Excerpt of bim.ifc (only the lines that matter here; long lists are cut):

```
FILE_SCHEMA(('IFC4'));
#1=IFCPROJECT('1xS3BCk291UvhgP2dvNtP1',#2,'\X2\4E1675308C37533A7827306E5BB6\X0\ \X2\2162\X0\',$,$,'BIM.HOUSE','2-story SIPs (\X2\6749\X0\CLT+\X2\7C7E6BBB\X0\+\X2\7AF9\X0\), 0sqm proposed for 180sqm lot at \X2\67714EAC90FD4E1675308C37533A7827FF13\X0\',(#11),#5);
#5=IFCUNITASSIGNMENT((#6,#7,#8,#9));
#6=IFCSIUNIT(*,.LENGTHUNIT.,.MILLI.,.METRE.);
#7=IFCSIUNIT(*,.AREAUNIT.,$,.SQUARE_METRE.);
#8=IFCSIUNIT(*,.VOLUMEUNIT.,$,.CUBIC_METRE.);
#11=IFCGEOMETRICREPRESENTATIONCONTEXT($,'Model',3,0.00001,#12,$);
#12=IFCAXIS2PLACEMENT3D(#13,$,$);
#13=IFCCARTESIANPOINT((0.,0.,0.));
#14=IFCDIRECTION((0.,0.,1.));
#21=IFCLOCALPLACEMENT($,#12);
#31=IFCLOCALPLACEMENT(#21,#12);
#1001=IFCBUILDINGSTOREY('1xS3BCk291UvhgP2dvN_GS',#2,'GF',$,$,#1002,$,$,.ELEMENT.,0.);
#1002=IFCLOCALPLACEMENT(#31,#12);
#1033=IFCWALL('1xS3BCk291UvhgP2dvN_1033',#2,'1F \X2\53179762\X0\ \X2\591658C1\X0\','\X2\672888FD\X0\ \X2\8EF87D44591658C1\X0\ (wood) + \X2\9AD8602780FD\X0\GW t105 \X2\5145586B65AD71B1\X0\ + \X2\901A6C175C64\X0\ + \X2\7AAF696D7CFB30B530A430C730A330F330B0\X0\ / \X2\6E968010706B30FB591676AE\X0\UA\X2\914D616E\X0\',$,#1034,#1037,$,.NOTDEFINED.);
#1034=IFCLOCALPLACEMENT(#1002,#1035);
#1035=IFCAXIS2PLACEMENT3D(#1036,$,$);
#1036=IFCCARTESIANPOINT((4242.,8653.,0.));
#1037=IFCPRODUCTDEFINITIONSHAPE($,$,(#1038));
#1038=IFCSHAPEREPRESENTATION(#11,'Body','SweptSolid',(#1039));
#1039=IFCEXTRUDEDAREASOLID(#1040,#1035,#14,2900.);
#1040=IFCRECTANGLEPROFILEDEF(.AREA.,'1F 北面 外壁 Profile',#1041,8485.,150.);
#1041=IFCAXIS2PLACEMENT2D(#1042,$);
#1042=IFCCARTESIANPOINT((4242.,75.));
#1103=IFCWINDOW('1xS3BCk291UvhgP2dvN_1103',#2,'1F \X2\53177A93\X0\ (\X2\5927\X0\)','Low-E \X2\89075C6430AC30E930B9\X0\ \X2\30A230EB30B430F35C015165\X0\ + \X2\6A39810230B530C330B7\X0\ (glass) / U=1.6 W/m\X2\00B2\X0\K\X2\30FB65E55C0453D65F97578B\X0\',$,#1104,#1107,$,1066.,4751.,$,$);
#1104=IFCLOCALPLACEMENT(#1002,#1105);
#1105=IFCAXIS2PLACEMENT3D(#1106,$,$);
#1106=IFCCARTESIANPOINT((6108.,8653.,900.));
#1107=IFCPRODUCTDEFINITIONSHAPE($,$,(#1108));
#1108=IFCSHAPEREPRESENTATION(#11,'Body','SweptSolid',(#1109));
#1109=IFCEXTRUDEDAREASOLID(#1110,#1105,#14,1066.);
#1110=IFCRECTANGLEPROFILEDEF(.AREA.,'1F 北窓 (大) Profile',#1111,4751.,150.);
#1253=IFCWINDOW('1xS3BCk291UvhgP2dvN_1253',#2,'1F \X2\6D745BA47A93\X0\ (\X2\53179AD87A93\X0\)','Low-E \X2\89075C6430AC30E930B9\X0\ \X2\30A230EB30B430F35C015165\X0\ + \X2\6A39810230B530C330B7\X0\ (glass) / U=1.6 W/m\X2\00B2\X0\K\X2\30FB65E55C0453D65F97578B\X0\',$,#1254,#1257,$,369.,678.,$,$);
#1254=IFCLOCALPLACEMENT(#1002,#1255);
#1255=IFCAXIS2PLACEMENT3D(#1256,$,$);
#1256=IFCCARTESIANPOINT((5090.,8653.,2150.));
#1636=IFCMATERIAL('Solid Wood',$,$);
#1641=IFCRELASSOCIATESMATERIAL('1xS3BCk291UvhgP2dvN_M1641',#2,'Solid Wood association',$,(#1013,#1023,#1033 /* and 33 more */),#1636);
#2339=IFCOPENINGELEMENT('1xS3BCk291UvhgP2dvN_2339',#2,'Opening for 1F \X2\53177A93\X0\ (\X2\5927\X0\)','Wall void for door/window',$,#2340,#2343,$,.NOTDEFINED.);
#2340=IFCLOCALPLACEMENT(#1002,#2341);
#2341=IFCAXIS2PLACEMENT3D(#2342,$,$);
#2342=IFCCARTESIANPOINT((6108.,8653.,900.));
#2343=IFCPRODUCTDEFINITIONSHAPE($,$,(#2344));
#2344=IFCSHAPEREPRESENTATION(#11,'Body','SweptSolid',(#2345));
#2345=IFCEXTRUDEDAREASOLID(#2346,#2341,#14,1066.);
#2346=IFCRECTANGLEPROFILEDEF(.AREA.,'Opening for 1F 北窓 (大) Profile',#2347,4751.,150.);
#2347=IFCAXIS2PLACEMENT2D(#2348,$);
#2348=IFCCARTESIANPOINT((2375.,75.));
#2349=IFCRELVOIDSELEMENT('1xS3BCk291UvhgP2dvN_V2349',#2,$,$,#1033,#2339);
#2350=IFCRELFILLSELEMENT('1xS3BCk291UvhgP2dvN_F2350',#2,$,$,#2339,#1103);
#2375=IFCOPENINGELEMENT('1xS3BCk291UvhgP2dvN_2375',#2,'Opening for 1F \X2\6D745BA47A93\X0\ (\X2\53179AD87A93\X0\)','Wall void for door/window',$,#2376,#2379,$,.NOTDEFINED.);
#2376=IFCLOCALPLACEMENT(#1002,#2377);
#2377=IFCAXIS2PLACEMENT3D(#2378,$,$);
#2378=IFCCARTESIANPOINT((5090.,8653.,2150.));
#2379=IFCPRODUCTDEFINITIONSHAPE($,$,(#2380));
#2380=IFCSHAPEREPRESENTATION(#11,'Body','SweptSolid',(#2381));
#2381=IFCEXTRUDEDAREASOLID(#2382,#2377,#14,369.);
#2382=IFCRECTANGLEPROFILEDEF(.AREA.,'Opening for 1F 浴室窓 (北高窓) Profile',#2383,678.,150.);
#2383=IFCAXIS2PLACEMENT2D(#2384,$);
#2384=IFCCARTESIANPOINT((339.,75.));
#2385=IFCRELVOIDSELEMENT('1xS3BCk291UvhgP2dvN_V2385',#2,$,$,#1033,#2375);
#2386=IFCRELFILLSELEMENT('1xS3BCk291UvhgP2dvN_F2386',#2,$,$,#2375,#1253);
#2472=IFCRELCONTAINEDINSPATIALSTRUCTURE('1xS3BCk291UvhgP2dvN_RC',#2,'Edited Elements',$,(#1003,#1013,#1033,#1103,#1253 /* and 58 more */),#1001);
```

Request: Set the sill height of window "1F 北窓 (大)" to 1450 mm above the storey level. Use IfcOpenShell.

```python
import numpy as np
import ifcopenshell
import ifcopenshell.api.geometry
import ifcopenshell.geom
import ifcopenshell.util.element
import ifcopenshell.util.placement
import ifcopenshell.util.shape
import ifcopenshell.util.unit

model = ifcopenshell.open("bim.ifc")
unit_scale = ifcopenshell.util.unit.calculate_unit_scale(model)

window = model.by_guid("1xS3BCk291UvhgP2dvN_1103")
opening = window.FillsVoids[0].RelatingOpeningElement
storey = ifcopenshell.util.element.get_container(window, ifc_class="IfcBuildingStorey")
level = ifcopenshell.util.placement.get_local_placement(storey.ObjectPlacement)[2, 3]

# The opening's origin need not be at the sill, so measure its lowest point.
shape = ifcopenshell.geom.create_shape(ifcopenshell.geom.settings(), opening)
bottom = ifcopenshell.util.shape.get_shape_bottom_elevation(shape, shape.geometry) / unit_scale
dz = level + 1.45 / unit_scale - bottom

shift = np.array([0.0, 0.0, dz])
# The window is not placed relative to its opening, so move both.
for product in (opening, window):
    matrix = ifcopenshell.util.placement.get_local_placement(product.ObjectPlacement)
    matrix[:3, 3] += shift
    ifcopenshell.api.geometry.edit_object_placement(model, product=product, matrix=matrix, is_si=False)

print(f"moved by {dz * unit_scale:+.3f} m")

model.write("bim_rev.ifc")
```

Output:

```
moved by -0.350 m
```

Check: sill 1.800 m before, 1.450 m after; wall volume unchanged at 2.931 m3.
